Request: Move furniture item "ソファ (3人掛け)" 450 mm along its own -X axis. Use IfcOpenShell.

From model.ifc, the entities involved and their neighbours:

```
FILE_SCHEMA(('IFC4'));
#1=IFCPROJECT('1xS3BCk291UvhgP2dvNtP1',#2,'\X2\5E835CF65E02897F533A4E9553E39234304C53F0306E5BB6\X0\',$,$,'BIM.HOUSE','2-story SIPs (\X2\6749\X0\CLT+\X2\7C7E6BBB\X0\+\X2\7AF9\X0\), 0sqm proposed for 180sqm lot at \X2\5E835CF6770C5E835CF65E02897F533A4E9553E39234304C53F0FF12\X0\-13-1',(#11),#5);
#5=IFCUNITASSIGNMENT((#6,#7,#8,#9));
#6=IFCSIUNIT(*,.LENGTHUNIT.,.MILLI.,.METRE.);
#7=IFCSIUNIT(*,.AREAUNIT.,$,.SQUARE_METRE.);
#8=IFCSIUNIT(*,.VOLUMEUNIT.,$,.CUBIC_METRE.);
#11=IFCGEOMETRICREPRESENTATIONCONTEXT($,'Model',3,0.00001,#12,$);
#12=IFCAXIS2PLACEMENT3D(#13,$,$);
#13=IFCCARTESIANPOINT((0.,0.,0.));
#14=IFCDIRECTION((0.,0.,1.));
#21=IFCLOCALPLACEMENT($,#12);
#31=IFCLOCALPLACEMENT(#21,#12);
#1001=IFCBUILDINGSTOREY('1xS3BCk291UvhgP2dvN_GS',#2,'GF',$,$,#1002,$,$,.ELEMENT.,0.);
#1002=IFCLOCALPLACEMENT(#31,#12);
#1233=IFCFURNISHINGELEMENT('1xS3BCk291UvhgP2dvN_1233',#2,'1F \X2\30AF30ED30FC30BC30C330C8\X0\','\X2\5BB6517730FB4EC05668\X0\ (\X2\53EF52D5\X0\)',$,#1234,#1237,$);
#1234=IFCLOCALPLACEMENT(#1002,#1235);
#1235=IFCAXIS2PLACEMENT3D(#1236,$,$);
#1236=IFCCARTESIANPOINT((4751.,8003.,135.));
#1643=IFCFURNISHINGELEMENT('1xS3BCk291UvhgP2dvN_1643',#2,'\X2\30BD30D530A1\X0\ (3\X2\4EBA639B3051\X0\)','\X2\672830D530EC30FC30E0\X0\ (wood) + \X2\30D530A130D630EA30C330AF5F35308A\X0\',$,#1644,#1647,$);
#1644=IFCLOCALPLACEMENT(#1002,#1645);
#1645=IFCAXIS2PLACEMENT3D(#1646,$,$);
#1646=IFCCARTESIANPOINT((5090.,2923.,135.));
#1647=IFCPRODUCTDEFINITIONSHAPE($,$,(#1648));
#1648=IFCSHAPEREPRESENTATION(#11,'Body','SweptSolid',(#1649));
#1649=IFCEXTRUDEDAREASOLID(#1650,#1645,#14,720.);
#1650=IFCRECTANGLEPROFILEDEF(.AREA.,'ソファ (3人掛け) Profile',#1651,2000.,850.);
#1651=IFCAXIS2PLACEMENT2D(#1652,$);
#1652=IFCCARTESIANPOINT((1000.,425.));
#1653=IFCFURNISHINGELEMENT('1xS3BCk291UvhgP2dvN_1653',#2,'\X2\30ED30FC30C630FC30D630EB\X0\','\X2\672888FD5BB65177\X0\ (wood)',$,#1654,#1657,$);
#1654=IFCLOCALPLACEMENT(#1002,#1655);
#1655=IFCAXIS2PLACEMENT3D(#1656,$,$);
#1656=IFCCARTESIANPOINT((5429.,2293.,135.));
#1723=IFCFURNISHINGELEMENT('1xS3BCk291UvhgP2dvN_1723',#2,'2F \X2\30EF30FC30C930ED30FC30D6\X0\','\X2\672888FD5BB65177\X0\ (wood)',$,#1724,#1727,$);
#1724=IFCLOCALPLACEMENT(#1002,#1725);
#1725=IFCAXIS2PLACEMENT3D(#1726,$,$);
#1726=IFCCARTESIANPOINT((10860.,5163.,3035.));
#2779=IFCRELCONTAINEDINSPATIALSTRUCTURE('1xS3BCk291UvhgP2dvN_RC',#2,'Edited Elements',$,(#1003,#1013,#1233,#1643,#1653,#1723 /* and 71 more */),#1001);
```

```python
import ifcopenshell
import ifcopenshell.api.geometry
import ifcopenshell.util.placement

model = ifcopenshell.open("model.ifc")

item = model.by_guid("1xS3BCk291UvhgP2dvN_1643")
matrix = ifcopenshell.util.placement.get_local_placement(item.ObjectPlacement)
matrix[:3, 3] -= matrix[:3, 0] * 450.0
ifcopenshell.api.geometry.edit_object_placement(model, product=item, matrix=matrix, is_si=False)

print(ifcopenshell.util.placement.get_local_placement(item.ObjectPlacement).round(3) + 0.0)

model.write("model-out.ifc")
```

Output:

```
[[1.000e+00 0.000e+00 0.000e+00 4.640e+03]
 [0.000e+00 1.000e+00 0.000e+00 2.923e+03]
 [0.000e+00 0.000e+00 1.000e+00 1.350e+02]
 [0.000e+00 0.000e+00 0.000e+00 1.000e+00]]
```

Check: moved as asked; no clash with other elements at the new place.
